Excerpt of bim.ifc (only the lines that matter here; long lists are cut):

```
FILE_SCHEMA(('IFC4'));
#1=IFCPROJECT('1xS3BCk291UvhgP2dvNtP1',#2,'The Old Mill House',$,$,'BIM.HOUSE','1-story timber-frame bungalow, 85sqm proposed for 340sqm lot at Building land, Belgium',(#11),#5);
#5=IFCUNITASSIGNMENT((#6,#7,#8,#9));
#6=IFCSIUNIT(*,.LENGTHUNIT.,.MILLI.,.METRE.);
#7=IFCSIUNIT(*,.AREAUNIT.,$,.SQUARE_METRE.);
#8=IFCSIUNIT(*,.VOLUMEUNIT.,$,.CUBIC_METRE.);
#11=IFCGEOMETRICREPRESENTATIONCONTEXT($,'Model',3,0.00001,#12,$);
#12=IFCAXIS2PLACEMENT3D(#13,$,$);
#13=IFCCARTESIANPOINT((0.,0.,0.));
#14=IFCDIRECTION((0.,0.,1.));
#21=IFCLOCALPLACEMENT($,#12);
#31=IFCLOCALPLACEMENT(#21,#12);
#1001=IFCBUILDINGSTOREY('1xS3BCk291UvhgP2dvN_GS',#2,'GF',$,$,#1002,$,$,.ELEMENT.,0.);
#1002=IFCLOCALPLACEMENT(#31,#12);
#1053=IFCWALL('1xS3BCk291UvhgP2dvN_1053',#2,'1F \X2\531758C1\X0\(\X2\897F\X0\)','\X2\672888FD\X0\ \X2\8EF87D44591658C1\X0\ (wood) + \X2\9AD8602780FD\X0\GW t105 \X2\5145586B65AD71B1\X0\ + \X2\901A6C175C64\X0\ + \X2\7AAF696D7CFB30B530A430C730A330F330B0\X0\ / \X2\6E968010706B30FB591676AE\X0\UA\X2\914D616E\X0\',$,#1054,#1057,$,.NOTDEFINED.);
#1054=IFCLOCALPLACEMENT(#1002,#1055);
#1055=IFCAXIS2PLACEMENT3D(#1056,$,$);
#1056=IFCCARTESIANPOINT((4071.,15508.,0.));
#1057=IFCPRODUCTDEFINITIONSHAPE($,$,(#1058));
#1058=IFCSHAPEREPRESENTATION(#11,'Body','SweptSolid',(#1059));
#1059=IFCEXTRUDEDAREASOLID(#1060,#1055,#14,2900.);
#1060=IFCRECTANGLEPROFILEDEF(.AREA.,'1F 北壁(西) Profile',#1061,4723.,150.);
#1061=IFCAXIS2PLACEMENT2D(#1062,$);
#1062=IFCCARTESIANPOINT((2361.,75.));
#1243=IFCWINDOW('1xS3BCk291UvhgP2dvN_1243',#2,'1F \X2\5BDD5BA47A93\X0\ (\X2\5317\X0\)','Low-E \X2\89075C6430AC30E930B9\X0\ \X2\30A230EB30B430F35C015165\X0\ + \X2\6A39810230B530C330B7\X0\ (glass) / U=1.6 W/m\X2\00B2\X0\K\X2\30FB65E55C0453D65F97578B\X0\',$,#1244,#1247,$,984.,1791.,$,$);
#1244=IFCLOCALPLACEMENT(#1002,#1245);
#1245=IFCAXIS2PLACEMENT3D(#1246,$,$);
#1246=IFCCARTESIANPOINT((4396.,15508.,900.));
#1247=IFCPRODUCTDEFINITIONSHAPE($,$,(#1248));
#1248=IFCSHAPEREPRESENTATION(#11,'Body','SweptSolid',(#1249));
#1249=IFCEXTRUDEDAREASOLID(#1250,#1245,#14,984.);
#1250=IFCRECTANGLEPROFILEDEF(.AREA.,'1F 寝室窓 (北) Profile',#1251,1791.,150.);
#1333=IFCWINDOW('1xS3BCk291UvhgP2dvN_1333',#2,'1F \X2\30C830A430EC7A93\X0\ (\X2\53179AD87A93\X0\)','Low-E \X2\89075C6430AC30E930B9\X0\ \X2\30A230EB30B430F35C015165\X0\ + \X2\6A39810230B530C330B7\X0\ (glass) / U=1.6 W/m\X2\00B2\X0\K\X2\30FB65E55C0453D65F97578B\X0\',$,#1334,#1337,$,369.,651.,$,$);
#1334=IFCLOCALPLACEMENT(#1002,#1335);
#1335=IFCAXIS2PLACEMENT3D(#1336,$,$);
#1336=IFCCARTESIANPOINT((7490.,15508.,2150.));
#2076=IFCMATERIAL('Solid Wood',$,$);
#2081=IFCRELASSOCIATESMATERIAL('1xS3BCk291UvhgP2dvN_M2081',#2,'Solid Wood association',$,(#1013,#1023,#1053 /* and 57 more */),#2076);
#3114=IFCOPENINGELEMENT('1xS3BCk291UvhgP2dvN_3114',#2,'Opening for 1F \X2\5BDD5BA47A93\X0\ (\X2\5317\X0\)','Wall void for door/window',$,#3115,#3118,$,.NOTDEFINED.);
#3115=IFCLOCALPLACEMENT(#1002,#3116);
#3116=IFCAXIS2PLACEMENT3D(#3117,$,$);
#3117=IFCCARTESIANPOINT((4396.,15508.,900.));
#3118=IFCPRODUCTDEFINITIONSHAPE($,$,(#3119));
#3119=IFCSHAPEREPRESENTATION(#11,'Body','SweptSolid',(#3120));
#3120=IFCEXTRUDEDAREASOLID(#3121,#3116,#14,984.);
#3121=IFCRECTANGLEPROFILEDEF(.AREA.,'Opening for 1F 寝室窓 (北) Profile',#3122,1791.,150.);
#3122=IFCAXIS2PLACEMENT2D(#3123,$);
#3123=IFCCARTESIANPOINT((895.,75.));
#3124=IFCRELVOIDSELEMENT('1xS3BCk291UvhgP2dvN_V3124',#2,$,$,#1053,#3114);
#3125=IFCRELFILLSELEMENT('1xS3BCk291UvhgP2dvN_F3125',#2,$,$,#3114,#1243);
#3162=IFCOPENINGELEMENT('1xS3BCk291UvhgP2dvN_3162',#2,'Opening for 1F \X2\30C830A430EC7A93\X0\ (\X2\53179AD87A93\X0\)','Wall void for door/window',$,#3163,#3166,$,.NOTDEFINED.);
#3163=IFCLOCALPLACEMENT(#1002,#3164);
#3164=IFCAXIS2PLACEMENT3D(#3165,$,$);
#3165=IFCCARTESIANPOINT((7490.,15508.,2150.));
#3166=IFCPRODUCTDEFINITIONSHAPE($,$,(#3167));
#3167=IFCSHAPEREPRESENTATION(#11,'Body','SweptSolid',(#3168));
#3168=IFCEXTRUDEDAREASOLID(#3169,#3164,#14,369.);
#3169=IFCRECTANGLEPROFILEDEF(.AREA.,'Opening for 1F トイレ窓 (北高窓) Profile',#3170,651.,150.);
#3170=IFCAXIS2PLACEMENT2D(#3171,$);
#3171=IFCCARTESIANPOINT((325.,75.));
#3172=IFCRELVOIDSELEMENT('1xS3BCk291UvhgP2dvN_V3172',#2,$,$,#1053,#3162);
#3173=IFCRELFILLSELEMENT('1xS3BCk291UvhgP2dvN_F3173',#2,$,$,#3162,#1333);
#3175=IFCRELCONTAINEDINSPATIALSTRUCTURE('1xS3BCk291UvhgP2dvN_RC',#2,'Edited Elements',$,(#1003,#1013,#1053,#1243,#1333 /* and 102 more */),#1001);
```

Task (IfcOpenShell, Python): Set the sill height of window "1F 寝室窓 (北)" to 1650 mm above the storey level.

```python
import numpy as np
import ifcopenshell
import ifcopenshell.api.geometry
import ifcopenshell.geom
import ifcopenshell.util.element
import ifcopenshell.util.placement
import ifcopenshell.util.shape
import ifcopenshell.util.unit

model = ifcopenshell.open("bim.ifc")
unit_scale = ifcopenshell.util.unit.calculate_unit_scale(model)

window = model.by_guid("1xS3BCk291UvhgP2dvN_1243")
opening = window.FillsVoids[0].RelatingOpeningElement
storey = ifcopenshell.util.element.get_container(window, ifc_class="IfcBuildingStorey")
level = ifcopenshell.util.placement.get_local_placement(storey.ObjectPlacement)[2, 3]

# The opening's origin need not be at the sill, so measure its lowest point.
shape = ifcopenshell.geom.create_shape(ifcopenshell.geom.settings(), opening)
bottom = ifcopenshell.util.shape.get_shape_bottom_elevation(shape, shape.geometry) / unit_scale
dz = level + 1650.0 - bottom

shift = np.array([0.0, 0.0, dz])
# The window is not placed relative to its opening, so move both.
for product in (opening, window):
    matrix = ifcopenshell.util.placement.get_local_placement(product.ObjectPlacement)
    matrix[:3, 3] += shift
    ifcopenshell.api.geometry.edit_object_placement(model, product=product, matrix=matrix, is_si=False)

print(f"moved by {dz * unit_scale:+.3f} m")

model.write("bim_v2.ifc")
```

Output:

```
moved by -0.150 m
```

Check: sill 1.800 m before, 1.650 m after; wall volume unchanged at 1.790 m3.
